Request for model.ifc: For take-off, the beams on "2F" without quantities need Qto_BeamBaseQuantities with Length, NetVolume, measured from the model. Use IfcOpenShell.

First a look at what the model holds.

```python
import ifcopenshell
import ifcopenshell.util.element
import ifcopenshell.util.unit

model = ifcopenshell.open("model.ifc")
print(model.schema)
for unit_type in ("LENGTHUNIT", "AREAUNIT", "VOLUMEUNIT"):
    print(unit_type, ifcopenshell.util.unit.calculate_unit_scale(model, unit_type))
storey = next(s for s in model.by_type("IfcBuildingStorey") if s.Name == "2F")
beams = [e for e in ifcopenshell.util.element.get_decomposition(storey) if e.is_a("IfcBeam")]
for e in sorted(beams, key=lambda e: e.id()):
    print(e.id(), e.is_a(), e.Name, list(ifcopenshell.util.element.get_psets(e, qtos_only=True)), sep=" | ")
```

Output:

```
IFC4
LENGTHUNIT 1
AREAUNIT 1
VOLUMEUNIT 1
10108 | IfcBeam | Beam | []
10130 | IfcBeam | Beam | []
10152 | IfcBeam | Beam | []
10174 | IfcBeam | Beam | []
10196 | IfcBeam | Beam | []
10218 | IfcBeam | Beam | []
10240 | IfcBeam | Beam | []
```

```python
import ifcopenshell
import ifcopenshell.api.pset
import ifcopenshell.geom
import ifcopenshell.util.element
import ifcopenshell.util.shape
import ifcopenshell.util.unit

model = ifcopenshell.open("model.ifc")
unit_scale = ifcopenshell.util.unit.calculate_unit_scale(model)
volume_scale = ifcopenshell.util.unit.calculate_unit_scale(model, "VOLUMEUNIT")
settings = ifcopenshell.geom.settings()

storey = next(s for s in model.by_type("IfcBuildingStorey") if s.Name == "2F")
beams = [e for e in ifcopenshell.util.element.get_decomposition(storey) if e.is_a("IfcBeam")]

for e in sorted(beams, key=lambda e: e.id()):
    if ifcopenshell.util.element.get_psets(e, qtos_only=True, should_inherit=False):
        continue
    # Geometry comes back in metres, in the element's own axes.
    shape = ifcopenshell.geom.create_shape(settings, e)
    values = {
        "Length": ifcopenshell.util.shape.get_max_xyz(shape.geometry) / unit_scale,
        "NetVolume": ifcopenshell.util.shape.get_volume(shape.geometry) / volume_scale,
    }
    qto = ifcopenshell.api.pset.add_qto(model, product=e, name="Qto_BeamBaseQuantities")
    ifcopenshell.api.pset.edit_qto(model, qto=qto, properties=values)
    print(e.id(), {k: round(v, 3) for k, v in values.items()})

model.write("model-out.ifc")
```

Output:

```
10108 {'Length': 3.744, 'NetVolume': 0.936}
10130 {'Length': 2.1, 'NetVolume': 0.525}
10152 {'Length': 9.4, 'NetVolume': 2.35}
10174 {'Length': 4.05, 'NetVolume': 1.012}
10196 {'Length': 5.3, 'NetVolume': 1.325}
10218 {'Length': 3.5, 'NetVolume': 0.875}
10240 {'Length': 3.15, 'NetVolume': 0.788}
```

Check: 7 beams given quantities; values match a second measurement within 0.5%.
